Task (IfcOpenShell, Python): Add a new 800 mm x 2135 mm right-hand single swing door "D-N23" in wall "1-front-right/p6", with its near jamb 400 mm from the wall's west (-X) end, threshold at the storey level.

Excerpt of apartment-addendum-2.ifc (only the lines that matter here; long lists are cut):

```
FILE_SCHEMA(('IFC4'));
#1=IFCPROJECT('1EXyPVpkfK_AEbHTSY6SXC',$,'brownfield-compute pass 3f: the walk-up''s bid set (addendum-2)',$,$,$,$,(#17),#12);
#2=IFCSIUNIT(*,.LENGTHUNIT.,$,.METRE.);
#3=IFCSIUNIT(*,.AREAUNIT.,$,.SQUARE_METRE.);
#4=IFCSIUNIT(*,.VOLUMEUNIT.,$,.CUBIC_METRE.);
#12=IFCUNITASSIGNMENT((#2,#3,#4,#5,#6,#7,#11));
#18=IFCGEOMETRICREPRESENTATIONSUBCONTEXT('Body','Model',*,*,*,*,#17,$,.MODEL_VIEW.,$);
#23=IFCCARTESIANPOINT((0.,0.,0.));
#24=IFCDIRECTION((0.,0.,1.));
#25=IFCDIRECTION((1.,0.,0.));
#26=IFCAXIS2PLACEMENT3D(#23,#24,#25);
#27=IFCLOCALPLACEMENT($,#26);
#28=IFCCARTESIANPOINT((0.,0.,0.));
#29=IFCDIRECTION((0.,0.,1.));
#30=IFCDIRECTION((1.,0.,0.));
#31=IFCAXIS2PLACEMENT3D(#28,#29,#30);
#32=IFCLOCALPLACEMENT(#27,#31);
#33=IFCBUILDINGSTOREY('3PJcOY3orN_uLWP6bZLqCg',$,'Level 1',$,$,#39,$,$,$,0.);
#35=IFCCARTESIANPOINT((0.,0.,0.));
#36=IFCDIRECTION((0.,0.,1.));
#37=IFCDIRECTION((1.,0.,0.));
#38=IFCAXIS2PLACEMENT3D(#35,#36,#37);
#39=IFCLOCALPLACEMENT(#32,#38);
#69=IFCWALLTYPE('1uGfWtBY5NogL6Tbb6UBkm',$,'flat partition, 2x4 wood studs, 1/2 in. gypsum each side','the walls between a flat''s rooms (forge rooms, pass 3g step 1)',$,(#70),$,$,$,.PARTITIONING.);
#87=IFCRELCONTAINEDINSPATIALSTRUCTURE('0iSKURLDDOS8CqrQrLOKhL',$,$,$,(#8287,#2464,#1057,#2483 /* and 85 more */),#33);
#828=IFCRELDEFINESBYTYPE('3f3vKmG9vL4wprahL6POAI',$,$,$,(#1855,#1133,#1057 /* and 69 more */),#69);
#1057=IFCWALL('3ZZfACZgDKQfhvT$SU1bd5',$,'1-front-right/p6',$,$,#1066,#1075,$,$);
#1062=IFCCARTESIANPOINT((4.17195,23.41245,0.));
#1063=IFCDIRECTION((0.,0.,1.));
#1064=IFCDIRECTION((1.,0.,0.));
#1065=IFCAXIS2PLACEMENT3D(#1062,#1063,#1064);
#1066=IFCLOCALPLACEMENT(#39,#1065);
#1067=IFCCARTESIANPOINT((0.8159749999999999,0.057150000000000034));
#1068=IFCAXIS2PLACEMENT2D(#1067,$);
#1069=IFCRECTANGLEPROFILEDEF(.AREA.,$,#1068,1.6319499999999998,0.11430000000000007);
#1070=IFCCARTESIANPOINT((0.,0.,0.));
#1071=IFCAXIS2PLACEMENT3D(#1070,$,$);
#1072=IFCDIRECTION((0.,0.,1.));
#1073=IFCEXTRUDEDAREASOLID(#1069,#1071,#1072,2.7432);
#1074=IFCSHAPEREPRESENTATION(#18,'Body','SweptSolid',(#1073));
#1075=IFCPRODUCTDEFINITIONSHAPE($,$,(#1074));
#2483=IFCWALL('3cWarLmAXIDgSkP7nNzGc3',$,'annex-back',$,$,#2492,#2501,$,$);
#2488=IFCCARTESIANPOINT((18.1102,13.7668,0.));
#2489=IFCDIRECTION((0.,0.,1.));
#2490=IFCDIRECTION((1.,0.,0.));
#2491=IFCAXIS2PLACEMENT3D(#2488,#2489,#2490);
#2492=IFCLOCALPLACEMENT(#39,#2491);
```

```python
import numpy as np
import ifcopenshell
import ifcopenshell.api.feature
import ifcopenshell.api.geometry
import ifcopenshell.api.root
import ifcopenshell.api.spatial
import ifcopenshell.geom
import ifcopenshell.util.element
import ifcopenshell.util.placement
import ifcopenshell.util.representation
import ifcopenshell.util.shape
import ifcopenshell.util.unit

model = ifcopenshell.open("apartment-addendum-2.ifc")
unit_scale = ifcopenshell.util.unit.calculate_unit_scale(model)
settings = ifcopenshell.geom.settings()


def volume(element):
    """Net volume in cubic metres, openings subtracted."""
    shape = ifcopenshell.geom.create_shape(settings, element)
    return ifcopenshell.util.shape.get_volume(shape.geometry)


wall = model.by_guid("3ZZfACZgDKQfhvT$SU1bd5")
storey = ifcopenshell.util.element.get_container(wall, ifc_class="IfcBuildingStorey")
context = ifcopenshell.util.representation.get_context(model, "Model", "Body", "MODEL_VIEW")
before = volume(wall)

width, height, from_end, sill = 0.8, 2.135, 0.4, 0.0  # metres

# The wall runs along its own X axis, and the end named is its -X end.
wall_shape = ifcopenshell.geom.create_shape(settings, wall)
x, y, z = ifcopenshell.util.shape.get_vertices(wall_shape.geometry).T
start = x.min() + from_end
face, thickness = float(y.min()), float(y.max() - y.min())
wall_matrix = ifcopenshell.util.placement.get_local_placement(wall.ObjectPlacement)
level = ifcopenshell.util.placement.get_local_placement(storey.ObjectPlacement)[2, 3]


def in_wall(x, y):
    """Placement at x, y metres in the wall's axes, at sill height."""
    matrix = wall_matrix.copy()
    matrix[:, 3] = wall_matrix @ np.array([x / unit_scale, y / unit_scale, 0.0, 1.0])
    matrix[2, 3] = level + sill / unit_scale
    return matrix


# Opening: a box that overshoots both wall faces by 50 mm.
opening = ifcopenshell.api.root.create_entity(model, ifc_class="IfcOpeningElement", predefined_type="OPENING")
box = ifcopenshell.api.geometry.add_wall_representation(
    model, context=context, length=width, height=height, thickness=thickness + 0.1
)
ifcopenshell.api.geometry.assign_representation(model, product=opening, representation=box)
ifcopenshell.api.geometry.edit_object_placement(model, product=opening, matrix=in_wall(start, face - 0.05), is_si=False)
ifcopenshell.api.feature.add_feature(model, feature=opening, element=wall)

door = ifcopenshell.api.root.create_entity(model, ifc_class="IfcDoor", name="D-N23", predefined_type="DOOR")
door.OverallWidth, door.OverallHeight = width / unit_scale, height / unit_scale
door.OperationType = "SINGLE_SWING_RIGHT"
body = ifcopenshell.api.geometry.add_door_representation(
    model,
    context=context,
    overall_width=door.OverallWidth,
    overall_height=door.OverallHeight,
    operation_type="SINGLE_SWING_RIGHT",
    lining_properties={"LiningDepth": thickness / unit_scale, "ThresholdDepth": thickness / unit_scale},
)
ifcopenshell.api.geometry.assign_representation(model, product=door, representation=body)
ifcopenshell.api.spatial.assign_container(model, products=[door], relating_structure=storey)
ifcopenshell.api.feature.add_filling(model, opening=opening, element=door)

# The lining spans the wall, so the door starts at the wall face.
ifcopenshell.api.geometry.edit_object_placement(model, product=door, matrix=in_wall(start, face), is_si=False)

after = volume(wall)

print(f"wall volume {before:.3f} -> {after:.3f} m3")

model.write("apartment-addendum-2-out.ifc")
```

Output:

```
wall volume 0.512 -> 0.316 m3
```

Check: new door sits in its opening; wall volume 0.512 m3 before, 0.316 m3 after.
